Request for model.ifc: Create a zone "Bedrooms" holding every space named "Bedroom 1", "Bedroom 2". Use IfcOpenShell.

First a look at what the model holds.

```python
import ifcopenshell

model = ifcopenshell.open("model.ifc")
print(model.schema)
seen = {}
for space in model.by_type("IfcSpace"):
    seen[space.LongName] = seen.get(space.LongName, 0) + 1
for name, count in sorted(seen.items(), key=str):
    print(count, "x", name)
print("zones:", [z.Name for z in model.by_type("IfcZone")][:20])
```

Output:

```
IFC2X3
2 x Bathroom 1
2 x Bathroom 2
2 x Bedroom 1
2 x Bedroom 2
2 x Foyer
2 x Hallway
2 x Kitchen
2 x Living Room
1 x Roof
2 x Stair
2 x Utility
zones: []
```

```python
import ifcopenshell
import ifcopenshell.api.group
import ifcopenshell.api.root

model = ifcopenshell.open("model.ifc")

names = {"Bedroom 1", "Bedroom 2"}
spaces = [s for s in model.by_type("IfcSpace") if s.LongName in names]

zone = ifcopenshell.api.root.create_entity(model, ifc_class="IfcZone", name="Bedrooms")
ifcopenshell.api.group.assign_group(model, products=spaces, group=zone)
print(len(spaces), "spaces in", zone.Name)

model.write("model_updated.ifc")
```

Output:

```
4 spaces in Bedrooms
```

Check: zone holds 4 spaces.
